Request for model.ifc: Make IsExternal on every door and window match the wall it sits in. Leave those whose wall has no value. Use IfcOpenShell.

First a look at what the model holds.

```python
import ifcopenshell
import ifcopenshell.util.element

model = ifcopenshell.open("model.ifc")
print(model.schema)
seen = {}
for e in model.by_type("IfcDoor") + model.by_type("IfcWindow"):
    if not e.FillsVoids:
        continue
    host = e.FillsVoids[0].RelatingOpeningElement.VoidsElements[0].RelatingBuildingElement
    own = ifcopenshell.util.element.get_pset(e, f"Pset_{e.is_a()[3:].removesuffix('StandardCase')}Common", "IsExternal")
    wall = ifcopenshell.util.element.get_pset(host, "Pset_WallCommon", "IsExternal")
    seen[e.is_a(), own, wall] = seen.get((e.is_a(), own, wall), 0) + 1
for (cls, own, wall), count in sorted(seen.items(), key=str):
    print(count, cls, "IsExternal:", own, "| host wall:", wall)
```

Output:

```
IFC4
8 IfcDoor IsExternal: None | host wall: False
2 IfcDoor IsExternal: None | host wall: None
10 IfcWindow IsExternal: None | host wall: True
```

```python
import ifcopenshell
import ifcopenshell.api.pset
import ifcopenshell.util.element

model = ifcopenshell.open("model.ifc")

count = 0
for ifc_class, pset_name in (("IfcDoor", "Pset_DoorCommon"), ("IfcWindow", "Pset_WindowCommon")):
    for e in model.by_type(ifc_class):
        if not e.FillsVoids:
            continue
        host = e.FillsVoids[0].RelatingOpeningElement.VoidsElements[0].RelatingBuildingElement
        external = ifcopenshell.util.element.get_pset(host, "Pset_WallCommon", "IsExternal")
        if external is None or ifcopenshell.util.element.get_pset(e, pset_name, "IsExternal") == external:
            continue
        pset = ifcopenshell.api.pset.add_pset(model, product=e, name=pset_name)
        ifcopenshell.api.pset.edit_pset(model, pset=pset, properties={"IsExternal": external})
        count += 1

print(count, "updated")

model.write("model_updated.ifc")
```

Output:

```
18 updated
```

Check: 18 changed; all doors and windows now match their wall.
